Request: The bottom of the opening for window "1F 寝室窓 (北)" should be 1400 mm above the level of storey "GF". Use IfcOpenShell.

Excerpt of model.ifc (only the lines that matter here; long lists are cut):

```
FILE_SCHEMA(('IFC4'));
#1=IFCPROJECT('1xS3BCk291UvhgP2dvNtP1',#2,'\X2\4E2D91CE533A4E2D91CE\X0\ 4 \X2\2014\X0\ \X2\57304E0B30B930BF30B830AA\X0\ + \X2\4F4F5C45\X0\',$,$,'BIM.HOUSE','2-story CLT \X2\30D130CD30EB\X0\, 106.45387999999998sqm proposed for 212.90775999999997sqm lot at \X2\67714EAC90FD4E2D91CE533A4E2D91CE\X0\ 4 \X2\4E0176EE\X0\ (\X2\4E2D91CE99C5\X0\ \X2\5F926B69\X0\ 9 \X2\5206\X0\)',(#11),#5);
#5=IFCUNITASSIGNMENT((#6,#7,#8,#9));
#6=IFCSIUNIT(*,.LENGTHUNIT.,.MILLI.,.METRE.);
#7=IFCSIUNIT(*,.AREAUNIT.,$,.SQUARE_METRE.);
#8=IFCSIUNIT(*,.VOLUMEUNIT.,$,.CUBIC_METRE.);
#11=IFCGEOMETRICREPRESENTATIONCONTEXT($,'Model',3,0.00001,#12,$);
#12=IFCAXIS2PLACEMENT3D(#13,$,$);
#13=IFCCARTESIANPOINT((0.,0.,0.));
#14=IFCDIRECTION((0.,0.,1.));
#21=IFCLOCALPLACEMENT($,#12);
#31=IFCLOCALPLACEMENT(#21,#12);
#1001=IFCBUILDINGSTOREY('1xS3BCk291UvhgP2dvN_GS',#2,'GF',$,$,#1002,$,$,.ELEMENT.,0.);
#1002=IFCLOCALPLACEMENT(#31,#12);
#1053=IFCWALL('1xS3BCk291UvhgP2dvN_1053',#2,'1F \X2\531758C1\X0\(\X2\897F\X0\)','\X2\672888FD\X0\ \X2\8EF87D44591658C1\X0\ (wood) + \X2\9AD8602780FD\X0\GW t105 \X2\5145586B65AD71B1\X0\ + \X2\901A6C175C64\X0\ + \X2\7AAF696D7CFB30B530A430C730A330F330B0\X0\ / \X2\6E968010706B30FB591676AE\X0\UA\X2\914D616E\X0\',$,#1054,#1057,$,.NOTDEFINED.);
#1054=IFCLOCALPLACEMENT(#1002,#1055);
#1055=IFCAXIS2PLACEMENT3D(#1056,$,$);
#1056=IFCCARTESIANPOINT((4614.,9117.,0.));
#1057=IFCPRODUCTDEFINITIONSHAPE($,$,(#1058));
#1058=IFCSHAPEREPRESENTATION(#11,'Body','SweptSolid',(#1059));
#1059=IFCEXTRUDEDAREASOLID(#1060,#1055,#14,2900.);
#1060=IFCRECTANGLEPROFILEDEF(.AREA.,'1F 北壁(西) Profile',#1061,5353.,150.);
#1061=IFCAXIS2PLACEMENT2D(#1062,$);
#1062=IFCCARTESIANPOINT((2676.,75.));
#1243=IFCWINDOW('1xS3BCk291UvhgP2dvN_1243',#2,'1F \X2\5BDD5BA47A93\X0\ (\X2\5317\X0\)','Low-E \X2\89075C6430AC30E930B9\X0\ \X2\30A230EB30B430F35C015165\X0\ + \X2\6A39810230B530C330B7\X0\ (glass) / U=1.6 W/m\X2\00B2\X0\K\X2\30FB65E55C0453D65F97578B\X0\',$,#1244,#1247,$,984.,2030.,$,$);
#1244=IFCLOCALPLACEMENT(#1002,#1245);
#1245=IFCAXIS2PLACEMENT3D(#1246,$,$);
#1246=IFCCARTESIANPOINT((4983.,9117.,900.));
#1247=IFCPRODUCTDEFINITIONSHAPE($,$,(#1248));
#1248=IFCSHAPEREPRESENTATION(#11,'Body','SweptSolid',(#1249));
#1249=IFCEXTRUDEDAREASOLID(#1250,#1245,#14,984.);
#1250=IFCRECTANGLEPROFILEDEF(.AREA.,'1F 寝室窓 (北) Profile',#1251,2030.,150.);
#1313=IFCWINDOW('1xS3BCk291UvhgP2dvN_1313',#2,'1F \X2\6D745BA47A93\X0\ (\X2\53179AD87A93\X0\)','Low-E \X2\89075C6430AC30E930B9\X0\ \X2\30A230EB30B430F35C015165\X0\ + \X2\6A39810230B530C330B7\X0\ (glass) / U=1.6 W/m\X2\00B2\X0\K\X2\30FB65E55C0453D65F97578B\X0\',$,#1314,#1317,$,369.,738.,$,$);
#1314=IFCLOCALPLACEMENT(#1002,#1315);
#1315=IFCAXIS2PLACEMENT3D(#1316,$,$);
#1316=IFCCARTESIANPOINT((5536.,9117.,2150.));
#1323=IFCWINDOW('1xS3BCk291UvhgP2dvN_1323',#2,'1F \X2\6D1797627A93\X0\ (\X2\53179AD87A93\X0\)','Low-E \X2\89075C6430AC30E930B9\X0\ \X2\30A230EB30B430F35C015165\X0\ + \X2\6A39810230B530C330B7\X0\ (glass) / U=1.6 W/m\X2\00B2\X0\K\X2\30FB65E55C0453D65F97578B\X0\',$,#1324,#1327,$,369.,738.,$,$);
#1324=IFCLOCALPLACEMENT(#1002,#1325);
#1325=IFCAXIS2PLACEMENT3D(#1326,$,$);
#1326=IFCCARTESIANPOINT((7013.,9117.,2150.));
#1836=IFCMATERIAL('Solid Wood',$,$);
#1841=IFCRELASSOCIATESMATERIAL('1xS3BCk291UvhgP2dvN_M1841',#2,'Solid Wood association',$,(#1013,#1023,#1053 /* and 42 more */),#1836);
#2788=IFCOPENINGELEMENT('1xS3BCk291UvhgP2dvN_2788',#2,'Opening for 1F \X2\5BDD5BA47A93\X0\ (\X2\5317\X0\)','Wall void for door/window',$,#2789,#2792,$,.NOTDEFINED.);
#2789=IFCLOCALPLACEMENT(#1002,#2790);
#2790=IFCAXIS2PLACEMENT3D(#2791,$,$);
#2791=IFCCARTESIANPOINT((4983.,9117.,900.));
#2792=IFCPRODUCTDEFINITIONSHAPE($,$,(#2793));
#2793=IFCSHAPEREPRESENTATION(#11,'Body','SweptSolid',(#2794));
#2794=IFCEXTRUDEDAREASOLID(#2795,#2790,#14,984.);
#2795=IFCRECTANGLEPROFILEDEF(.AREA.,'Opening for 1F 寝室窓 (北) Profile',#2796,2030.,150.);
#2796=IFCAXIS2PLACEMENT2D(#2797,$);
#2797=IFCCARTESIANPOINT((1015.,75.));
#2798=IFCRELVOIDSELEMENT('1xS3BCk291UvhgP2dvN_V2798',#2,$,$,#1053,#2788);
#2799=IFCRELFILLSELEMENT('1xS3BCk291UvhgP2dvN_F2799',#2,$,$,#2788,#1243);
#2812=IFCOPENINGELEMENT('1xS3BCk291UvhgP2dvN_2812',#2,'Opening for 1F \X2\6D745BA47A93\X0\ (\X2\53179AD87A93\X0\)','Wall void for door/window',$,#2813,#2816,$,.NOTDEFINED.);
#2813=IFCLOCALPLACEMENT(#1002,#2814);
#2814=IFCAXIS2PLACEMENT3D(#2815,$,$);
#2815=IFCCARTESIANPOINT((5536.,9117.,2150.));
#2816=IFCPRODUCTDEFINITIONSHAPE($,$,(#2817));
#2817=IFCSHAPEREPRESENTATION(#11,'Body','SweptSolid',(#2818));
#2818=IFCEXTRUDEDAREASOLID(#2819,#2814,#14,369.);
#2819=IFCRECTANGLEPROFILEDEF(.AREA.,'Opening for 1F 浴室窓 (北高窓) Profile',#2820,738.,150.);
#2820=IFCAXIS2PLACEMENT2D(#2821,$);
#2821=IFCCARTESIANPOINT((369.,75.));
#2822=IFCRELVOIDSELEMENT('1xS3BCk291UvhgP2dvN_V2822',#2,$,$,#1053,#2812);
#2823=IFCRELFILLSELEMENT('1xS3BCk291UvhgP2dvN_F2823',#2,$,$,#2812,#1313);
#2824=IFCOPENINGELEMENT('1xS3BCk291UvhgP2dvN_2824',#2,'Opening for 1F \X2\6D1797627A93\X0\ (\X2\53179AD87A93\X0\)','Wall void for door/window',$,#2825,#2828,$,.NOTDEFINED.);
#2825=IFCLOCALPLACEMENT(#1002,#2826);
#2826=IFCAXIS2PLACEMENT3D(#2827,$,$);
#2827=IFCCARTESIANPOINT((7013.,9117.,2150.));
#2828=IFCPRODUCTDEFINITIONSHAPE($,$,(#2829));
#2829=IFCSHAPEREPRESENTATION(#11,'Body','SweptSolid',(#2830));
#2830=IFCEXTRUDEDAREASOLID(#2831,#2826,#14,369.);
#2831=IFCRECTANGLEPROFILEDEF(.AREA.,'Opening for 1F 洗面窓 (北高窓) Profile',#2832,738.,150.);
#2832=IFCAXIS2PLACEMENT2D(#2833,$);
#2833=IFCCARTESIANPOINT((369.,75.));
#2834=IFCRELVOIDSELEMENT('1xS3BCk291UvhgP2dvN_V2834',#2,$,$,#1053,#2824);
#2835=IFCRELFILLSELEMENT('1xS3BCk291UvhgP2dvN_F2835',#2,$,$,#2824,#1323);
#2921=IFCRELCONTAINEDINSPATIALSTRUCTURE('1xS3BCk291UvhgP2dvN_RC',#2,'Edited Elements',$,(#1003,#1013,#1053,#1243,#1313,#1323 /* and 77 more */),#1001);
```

```python
import numpy as np
import ifcopenshell
import ifcopenshell.api.geometry
import ifcopenshell.geom
import ifcopenshell.util.element
import ifcopenshell.util.placement
import ifcopenshell.util.shape
import ifcopenshell.util.unit

model = ifcopenshell.open("model.ifc")
unit_scale = ifcopenshell.util.unit.calculate_unit_scale(model)

window = model.by_guid("1xS3BCk291UvhgP2dvN_1243")
opening = window.FillsVoids[0].RelatingOpeningElement
storey = ifcopenshell.util.element.get_container(window, ifc_class="IfcBuildingStorey")
level = ifcopenshell.util.placement.get_local_placement(storey.ObjectPlacement)[2, 3]

# The opening's origin need not be at the sill, so measure its lowest point.
shape = ifcopenshell.geom.create_shape(ifcopenshell.geom.settings(), opening)
bottom = ifcopenshell.util.shape.get_shape_bottom_elevation(shape, shape.geometry) / unit_scale
dz = level + 1400.0 - bottom

shift = np.array([0.0, 0.0, dz])
# The window is not placed relative to its opening, so move both.
for product in (opening, window):
    matrix = ifcopenshell.util.placement.get_local_placement(product.ObjectPlacement)
    matrix[:3, 3] += shift
    ifcopenshell.api.geometry.edit_object_placement(model, product=product, matrix=matrix, is_si=False)

print(f"moved by {dz * unit_scale:+.3f} m")

model.write("model_rev.ifc")
```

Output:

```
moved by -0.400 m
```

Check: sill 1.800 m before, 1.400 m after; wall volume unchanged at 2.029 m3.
